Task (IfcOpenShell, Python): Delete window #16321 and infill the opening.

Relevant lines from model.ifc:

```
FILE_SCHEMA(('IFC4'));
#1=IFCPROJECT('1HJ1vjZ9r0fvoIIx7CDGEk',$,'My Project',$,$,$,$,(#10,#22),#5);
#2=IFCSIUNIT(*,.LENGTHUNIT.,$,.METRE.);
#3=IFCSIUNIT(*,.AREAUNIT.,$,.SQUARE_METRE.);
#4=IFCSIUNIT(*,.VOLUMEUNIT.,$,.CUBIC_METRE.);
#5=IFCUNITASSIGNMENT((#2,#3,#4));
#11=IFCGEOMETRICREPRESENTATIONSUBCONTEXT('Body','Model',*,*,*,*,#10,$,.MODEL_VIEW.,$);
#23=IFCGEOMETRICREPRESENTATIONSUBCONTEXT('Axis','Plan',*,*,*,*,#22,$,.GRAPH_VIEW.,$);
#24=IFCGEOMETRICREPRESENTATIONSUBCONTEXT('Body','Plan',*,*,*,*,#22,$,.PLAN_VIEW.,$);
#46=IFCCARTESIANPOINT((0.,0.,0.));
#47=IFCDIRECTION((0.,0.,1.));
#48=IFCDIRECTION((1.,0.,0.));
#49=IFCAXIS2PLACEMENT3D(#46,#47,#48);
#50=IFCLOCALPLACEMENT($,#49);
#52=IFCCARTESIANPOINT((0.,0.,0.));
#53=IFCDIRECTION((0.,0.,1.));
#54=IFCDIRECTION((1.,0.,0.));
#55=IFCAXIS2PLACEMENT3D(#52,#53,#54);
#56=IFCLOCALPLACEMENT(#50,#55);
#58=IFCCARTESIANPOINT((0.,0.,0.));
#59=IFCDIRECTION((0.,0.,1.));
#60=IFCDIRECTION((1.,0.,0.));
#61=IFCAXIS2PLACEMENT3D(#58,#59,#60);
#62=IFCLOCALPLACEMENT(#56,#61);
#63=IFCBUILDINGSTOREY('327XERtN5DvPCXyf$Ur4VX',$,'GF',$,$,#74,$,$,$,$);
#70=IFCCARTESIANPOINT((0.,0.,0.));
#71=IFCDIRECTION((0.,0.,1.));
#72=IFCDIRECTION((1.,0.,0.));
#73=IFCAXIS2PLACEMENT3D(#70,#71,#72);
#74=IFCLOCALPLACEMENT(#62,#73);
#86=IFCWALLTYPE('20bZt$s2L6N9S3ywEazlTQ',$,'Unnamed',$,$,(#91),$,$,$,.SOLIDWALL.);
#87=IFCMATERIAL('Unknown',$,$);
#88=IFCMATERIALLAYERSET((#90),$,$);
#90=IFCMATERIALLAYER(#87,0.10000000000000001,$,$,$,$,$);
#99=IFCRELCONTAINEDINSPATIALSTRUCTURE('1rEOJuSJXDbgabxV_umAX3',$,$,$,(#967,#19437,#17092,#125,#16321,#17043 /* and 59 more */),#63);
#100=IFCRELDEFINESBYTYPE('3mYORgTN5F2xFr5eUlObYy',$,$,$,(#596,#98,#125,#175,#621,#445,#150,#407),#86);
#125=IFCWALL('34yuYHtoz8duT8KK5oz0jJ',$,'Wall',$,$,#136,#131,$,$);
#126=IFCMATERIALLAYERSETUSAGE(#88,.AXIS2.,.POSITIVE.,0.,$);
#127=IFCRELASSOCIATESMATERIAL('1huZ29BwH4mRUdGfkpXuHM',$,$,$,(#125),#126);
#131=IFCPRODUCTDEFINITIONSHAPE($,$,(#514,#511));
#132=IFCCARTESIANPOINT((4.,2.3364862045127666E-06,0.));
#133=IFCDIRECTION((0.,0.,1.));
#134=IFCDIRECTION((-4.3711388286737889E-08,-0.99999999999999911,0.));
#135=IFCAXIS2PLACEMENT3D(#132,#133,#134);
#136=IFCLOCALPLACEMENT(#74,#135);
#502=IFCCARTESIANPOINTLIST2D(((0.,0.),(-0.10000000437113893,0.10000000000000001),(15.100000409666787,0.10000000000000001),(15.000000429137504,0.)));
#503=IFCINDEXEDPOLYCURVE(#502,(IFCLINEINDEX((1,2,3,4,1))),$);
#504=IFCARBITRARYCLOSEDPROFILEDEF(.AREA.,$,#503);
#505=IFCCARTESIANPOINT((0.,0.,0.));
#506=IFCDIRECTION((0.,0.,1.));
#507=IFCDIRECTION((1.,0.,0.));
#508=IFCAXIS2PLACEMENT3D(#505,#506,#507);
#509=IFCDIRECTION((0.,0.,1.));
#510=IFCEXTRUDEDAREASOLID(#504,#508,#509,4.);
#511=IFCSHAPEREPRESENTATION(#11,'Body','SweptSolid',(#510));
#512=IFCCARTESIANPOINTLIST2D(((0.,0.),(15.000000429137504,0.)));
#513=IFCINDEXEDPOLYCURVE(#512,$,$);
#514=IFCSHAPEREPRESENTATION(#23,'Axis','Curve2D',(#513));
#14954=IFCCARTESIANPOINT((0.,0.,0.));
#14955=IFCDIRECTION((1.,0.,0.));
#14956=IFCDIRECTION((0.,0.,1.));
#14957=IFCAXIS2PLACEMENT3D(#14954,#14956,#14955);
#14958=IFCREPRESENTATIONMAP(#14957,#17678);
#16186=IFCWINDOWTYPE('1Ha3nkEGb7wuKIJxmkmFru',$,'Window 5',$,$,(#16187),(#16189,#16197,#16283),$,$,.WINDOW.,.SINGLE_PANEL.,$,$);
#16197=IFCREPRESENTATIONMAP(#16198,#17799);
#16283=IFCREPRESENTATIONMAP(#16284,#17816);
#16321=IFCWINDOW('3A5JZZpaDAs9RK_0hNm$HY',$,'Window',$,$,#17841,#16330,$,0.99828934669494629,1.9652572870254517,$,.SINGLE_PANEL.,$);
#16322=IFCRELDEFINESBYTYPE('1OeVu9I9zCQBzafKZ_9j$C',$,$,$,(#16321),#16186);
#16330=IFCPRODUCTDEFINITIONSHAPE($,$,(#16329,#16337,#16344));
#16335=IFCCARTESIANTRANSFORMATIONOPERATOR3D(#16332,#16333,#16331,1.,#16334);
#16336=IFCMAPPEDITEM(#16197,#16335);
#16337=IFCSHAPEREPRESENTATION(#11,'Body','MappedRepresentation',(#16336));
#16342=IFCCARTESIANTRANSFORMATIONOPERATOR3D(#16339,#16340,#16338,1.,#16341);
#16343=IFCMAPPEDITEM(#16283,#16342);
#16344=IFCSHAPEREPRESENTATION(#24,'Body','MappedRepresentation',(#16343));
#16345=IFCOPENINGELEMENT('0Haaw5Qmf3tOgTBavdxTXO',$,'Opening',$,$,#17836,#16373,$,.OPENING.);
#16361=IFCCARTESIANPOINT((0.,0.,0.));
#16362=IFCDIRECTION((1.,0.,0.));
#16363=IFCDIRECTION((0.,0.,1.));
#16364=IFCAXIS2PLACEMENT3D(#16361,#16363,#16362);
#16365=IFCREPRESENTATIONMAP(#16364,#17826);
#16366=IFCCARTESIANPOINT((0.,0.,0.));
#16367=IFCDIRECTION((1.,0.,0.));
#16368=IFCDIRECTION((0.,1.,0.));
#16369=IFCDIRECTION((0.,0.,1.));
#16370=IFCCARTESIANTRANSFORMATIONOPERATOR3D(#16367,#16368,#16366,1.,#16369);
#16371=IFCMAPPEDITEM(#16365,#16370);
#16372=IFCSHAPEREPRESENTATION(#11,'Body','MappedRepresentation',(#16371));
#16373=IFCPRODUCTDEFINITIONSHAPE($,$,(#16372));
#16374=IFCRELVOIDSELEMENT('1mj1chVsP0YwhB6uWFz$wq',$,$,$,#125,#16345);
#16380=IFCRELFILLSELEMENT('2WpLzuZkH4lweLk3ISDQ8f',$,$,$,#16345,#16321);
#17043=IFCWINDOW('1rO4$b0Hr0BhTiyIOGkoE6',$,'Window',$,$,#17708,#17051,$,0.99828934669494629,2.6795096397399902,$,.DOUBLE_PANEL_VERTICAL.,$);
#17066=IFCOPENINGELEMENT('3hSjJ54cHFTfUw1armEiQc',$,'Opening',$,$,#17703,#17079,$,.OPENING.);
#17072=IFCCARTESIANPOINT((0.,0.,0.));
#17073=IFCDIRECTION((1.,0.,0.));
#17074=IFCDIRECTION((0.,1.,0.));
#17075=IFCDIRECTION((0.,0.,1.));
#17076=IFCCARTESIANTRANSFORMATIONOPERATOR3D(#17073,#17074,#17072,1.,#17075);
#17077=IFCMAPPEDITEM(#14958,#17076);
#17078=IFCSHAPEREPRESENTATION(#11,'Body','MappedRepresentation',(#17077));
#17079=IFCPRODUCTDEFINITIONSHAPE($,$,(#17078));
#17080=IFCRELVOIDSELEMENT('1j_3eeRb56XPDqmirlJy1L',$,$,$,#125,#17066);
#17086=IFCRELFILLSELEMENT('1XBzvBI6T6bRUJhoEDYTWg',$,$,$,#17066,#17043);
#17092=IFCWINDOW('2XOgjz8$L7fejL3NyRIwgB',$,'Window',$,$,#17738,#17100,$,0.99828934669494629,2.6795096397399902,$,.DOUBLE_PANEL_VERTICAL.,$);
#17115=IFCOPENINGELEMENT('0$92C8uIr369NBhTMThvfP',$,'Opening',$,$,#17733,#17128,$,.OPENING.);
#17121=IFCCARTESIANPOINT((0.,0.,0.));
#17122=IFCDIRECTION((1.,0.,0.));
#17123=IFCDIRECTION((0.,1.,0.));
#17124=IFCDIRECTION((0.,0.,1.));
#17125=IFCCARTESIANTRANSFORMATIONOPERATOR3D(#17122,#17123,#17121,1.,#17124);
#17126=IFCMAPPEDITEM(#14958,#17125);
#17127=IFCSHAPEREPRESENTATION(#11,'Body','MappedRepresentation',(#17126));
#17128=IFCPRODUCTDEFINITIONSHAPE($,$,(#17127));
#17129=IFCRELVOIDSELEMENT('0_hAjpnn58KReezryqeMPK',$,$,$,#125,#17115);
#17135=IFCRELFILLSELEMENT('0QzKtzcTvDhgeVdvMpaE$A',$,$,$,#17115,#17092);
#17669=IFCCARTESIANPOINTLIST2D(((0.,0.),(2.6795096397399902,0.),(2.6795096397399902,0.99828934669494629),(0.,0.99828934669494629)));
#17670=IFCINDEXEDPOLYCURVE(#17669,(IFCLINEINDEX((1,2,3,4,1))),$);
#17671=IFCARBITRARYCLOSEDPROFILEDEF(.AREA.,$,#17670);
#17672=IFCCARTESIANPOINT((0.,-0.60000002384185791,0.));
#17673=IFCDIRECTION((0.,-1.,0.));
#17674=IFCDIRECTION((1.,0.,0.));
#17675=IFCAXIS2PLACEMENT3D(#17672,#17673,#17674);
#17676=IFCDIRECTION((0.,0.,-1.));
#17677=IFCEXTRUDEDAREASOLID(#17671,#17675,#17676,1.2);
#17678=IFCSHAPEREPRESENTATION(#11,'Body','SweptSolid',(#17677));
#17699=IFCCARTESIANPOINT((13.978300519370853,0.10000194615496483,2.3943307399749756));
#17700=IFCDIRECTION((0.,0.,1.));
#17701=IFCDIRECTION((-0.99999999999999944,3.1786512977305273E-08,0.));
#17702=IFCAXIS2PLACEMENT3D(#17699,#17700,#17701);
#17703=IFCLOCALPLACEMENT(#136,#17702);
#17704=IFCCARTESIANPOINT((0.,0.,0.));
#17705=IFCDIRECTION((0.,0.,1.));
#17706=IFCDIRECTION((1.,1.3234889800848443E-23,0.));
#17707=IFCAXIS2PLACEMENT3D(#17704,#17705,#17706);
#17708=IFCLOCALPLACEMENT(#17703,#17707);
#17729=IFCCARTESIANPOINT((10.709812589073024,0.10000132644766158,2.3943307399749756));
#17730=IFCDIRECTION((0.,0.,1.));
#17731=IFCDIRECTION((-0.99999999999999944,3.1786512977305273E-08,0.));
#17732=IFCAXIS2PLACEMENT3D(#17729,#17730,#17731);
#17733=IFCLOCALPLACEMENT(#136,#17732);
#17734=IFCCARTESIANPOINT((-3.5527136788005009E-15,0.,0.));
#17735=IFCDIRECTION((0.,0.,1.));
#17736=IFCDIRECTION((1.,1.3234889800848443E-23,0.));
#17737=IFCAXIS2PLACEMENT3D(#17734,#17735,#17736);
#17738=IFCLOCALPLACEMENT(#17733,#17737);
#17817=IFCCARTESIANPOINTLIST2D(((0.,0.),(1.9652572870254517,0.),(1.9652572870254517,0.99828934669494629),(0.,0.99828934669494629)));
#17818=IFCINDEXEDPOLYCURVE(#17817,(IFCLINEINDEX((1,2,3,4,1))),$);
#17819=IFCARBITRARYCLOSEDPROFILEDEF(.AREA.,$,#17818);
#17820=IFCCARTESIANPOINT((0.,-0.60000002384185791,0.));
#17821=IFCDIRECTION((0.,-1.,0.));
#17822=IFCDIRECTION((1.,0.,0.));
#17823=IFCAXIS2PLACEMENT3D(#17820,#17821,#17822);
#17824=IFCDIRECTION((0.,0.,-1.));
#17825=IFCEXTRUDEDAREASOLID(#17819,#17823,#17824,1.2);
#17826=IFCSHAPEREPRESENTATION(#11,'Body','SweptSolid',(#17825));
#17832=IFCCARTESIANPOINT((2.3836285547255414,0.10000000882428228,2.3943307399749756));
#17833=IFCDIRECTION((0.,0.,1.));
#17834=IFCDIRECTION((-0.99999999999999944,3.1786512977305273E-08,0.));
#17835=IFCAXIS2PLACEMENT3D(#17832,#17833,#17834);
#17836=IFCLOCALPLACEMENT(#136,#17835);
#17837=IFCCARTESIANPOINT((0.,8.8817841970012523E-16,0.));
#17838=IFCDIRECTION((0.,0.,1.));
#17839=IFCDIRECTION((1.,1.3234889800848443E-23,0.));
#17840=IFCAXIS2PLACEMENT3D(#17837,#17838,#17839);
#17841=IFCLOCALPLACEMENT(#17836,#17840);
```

```python
import ifcopenshell
import ifcopenshell.api.feature
import ifcopenshell.api.root
import ifcopenshell.geom
import ifcopenshell.util.shape

model = ifcopenshell.open("model.ifc")
settings = ifcopenshell.geom.settings()


def volume(element):
    """Net volume in cubic metres, openings subtracted."""
    shape = ifcopenshell.geom.create_shape(settings, element)
    return ifcopenshell.util.shape.get_volume(shape.geometry)


window = model.by_guid("3A5JZZpaDAs9RK_0hNm$HY")
opening = window.FillsVoids[0].RelatingOpeningElement
wall = opening.VoidsElements[0].RelatingBuildingElement
before = volume(wall)

ifcopenshell.api.root.remove_product(model, product=window)
ifcopenshell.api.feature.remove_feature(model, feature=opening)

after = volume(wall)

print(f"wall volume {before:.3f} -> {after:.3f} m3")

model.write("model_updated.ifc")
```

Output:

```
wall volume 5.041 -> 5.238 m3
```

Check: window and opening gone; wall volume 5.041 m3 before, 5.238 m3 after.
